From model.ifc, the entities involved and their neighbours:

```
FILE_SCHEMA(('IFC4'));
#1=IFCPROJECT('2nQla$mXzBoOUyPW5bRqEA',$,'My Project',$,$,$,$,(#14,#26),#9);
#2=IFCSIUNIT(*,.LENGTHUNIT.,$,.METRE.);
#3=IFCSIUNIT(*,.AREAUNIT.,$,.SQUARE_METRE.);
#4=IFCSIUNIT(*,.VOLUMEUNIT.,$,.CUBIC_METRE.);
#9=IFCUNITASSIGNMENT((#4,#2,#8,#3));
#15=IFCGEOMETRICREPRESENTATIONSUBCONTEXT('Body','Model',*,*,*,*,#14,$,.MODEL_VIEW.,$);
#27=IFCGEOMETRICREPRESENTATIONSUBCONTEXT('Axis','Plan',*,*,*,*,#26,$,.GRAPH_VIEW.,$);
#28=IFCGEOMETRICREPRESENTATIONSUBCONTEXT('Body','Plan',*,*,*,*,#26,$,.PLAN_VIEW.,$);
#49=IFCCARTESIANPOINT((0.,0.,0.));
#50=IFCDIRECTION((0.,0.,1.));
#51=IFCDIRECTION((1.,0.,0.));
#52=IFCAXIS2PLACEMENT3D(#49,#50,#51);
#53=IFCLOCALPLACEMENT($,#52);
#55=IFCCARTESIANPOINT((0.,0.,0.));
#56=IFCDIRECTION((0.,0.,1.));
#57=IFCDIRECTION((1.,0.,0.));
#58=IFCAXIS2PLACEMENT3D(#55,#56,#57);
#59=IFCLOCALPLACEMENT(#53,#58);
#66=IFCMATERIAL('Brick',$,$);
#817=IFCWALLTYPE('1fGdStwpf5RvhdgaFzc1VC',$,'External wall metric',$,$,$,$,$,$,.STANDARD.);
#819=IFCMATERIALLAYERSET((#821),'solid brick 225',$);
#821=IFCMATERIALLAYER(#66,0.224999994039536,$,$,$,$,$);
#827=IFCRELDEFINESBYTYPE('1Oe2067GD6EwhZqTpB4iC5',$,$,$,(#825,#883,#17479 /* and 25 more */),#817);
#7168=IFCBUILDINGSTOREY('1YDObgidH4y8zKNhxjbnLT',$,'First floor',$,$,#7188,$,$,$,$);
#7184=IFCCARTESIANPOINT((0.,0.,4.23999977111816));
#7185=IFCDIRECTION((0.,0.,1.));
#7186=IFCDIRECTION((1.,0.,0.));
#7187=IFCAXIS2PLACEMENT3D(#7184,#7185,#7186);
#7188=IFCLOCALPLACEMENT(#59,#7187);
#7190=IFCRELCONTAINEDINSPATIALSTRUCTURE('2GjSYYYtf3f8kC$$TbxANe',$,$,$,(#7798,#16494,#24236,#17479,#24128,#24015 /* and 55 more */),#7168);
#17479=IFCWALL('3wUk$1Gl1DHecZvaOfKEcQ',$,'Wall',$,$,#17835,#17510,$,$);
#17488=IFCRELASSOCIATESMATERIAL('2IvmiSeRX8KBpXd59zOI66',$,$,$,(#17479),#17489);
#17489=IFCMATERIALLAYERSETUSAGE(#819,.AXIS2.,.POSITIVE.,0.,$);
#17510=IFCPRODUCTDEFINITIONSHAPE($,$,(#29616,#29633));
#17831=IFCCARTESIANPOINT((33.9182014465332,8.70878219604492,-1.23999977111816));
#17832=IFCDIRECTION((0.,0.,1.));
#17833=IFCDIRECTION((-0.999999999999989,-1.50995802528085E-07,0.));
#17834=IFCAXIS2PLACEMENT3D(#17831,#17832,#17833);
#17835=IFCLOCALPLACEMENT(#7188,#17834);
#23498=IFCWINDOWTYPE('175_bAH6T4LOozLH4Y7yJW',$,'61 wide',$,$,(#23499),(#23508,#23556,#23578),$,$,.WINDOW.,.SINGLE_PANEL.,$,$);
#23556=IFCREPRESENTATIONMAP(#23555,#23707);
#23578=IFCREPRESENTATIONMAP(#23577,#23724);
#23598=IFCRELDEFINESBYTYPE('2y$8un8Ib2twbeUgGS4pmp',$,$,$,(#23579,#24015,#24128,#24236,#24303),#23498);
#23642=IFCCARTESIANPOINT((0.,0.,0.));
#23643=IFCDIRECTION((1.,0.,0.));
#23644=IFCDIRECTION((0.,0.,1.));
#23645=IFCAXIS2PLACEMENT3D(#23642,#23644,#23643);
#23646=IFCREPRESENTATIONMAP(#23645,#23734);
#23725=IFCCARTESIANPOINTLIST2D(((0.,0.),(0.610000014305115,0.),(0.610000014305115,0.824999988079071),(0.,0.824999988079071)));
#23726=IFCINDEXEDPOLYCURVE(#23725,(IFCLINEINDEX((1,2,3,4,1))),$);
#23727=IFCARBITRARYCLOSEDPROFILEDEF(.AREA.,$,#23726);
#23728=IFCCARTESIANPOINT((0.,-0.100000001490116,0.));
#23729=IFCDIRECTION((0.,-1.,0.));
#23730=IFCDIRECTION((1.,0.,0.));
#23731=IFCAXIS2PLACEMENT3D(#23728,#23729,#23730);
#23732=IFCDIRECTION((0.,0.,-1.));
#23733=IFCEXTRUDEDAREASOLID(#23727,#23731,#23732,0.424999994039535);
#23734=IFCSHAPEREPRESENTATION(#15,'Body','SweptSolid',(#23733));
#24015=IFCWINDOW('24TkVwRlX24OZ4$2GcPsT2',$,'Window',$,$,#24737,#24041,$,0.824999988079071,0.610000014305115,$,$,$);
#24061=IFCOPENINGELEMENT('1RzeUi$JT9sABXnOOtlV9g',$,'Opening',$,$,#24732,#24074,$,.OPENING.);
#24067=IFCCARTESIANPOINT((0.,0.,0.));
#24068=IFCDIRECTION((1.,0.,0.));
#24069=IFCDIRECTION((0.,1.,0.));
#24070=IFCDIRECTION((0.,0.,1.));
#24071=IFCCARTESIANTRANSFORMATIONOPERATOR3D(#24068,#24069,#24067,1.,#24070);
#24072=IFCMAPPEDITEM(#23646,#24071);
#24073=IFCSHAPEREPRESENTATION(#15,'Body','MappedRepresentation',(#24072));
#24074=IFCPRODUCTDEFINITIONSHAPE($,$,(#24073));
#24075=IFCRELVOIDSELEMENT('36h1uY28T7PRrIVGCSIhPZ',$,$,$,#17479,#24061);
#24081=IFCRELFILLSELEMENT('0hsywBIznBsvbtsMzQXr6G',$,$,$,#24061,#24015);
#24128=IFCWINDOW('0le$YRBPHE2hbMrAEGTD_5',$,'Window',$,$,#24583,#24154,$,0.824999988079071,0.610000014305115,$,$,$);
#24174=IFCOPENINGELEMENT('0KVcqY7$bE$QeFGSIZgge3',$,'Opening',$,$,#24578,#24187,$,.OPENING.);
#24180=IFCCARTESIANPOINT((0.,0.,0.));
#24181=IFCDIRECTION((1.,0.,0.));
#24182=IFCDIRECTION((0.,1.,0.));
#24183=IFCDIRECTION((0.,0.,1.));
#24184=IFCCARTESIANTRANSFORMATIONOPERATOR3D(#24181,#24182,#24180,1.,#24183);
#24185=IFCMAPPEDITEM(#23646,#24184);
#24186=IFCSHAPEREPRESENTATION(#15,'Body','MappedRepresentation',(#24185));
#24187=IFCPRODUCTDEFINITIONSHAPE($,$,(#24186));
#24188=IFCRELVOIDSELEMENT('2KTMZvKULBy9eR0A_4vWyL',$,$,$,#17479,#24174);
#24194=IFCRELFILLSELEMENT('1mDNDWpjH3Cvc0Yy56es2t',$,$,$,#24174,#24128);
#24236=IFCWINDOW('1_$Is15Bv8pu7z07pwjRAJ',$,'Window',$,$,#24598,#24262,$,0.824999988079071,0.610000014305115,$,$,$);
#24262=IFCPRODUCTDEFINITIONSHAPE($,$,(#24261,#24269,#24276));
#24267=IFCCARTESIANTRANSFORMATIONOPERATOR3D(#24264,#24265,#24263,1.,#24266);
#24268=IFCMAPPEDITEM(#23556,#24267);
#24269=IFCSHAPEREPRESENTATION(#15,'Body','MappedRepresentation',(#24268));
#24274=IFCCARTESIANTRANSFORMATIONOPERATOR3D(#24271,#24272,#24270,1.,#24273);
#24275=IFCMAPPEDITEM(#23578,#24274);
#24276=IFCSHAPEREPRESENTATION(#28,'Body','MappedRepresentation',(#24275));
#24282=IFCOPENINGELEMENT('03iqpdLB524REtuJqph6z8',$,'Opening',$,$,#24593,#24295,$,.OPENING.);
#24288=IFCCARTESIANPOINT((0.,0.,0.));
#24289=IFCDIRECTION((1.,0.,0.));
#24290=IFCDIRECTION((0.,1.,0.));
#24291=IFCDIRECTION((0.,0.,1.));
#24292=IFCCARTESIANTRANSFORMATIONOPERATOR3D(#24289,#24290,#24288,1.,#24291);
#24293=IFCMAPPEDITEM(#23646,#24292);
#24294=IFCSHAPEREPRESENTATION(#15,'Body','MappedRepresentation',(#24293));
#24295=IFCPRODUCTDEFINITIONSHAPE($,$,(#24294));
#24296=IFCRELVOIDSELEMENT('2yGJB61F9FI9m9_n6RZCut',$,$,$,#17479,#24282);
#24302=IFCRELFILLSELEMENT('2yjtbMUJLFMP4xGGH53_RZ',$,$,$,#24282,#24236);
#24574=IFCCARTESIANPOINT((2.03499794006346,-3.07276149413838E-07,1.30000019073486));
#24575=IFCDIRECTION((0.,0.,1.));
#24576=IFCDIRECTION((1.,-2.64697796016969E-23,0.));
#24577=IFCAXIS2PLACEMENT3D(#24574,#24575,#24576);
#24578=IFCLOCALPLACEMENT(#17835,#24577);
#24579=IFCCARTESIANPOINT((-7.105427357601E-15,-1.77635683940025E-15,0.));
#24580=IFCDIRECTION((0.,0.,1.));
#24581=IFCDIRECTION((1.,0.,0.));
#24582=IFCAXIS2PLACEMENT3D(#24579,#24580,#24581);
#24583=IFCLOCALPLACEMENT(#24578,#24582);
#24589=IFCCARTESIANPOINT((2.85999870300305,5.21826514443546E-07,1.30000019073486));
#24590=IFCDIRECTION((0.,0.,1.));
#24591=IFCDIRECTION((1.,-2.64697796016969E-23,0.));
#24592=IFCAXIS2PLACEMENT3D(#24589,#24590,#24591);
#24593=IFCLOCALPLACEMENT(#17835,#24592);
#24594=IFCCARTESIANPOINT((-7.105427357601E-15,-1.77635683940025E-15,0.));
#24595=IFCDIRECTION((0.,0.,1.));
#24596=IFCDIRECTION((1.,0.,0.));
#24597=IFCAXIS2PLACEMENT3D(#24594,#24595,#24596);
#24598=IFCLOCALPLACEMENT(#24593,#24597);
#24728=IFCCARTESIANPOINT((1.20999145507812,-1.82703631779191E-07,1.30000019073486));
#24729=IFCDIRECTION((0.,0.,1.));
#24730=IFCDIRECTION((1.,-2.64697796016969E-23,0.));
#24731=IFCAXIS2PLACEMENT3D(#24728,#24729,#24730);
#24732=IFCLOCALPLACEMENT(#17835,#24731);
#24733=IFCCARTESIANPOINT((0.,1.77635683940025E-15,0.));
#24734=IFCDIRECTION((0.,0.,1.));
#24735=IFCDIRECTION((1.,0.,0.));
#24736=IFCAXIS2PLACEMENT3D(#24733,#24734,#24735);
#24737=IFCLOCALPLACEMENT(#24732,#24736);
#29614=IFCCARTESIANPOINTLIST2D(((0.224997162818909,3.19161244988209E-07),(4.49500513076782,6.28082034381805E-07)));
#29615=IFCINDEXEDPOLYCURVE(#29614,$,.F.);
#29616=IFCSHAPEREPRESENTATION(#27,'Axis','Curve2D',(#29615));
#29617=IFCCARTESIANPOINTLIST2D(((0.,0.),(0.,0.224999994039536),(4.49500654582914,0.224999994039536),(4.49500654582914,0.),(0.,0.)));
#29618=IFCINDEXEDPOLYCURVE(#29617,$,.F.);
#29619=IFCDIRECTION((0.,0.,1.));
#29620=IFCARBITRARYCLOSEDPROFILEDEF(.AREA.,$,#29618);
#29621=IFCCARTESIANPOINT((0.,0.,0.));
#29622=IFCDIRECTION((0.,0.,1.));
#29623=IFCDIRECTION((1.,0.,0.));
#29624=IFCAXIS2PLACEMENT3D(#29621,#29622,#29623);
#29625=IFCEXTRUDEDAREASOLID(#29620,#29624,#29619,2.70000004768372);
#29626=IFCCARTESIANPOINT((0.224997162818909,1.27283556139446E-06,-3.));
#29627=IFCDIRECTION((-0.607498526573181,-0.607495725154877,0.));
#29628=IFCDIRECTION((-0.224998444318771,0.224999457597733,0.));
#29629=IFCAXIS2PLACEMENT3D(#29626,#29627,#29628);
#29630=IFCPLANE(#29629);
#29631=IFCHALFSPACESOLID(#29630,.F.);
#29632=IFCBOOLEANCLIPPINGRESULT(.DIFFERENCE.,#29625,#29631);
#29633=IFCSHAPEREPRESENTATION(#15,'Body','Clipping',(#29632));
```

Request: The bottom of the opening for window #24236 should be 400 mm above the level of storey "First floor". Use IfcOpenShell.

```python
import numpy as np
import ifcopenshell
import ifcopenshell.api.geometry
import ifcopenshell.geom
import ifcopenshell.util.element
import ifcopenshell.util.placement
import ifcopenshell.util.shape
import ifcopenshell.util.unit

model = ifcopenshell.open("model.ifc")
unit_scale = ifcopenshell.util.unit.calculate_unit_scale(model)

window = model.by_id(24236)
opening = window.FillsVoids[0].RelatingOpeningElement
storey = ifcopenshell.util.element.get_container(window, ifc_class="IfcBuildingStorey")
level = ifcopenshell.util.placement.get_local_placement(storey.ObjectPlacement)[2, 3]

# The opening's origin need not be at the sill, so measure its lowest point.
shape = ifcopenshell.geom.create_shape(ifcopenshell.geom.settings(), opening)
bottom = ifcopenshell.util.shape.get_shape_bottom_elevation(shape, shape.geometry) / unit_scale
dz = level + 0.4 - bottom

shift = np.array([0.0, 0.0, dz])
# The window is placed relative to its opening, so it follows when the opening moves.
matrix = ifcopenshell.util.placement.get_local_placement(opening.ObjectPlacement)
matrix[:3, 3] += shift
ifcopenshell.api.geometry.edit_object_placement(
    model, product=opening, matrix=matrix, is_si=False, should_transform_children=True
)

print(f"moved by {dz * unit_scale:+.3f} m")

model.write("model_edited.ifc")
```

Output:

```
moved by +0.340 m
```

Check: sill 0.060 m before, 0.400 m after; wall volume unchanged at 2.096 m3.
